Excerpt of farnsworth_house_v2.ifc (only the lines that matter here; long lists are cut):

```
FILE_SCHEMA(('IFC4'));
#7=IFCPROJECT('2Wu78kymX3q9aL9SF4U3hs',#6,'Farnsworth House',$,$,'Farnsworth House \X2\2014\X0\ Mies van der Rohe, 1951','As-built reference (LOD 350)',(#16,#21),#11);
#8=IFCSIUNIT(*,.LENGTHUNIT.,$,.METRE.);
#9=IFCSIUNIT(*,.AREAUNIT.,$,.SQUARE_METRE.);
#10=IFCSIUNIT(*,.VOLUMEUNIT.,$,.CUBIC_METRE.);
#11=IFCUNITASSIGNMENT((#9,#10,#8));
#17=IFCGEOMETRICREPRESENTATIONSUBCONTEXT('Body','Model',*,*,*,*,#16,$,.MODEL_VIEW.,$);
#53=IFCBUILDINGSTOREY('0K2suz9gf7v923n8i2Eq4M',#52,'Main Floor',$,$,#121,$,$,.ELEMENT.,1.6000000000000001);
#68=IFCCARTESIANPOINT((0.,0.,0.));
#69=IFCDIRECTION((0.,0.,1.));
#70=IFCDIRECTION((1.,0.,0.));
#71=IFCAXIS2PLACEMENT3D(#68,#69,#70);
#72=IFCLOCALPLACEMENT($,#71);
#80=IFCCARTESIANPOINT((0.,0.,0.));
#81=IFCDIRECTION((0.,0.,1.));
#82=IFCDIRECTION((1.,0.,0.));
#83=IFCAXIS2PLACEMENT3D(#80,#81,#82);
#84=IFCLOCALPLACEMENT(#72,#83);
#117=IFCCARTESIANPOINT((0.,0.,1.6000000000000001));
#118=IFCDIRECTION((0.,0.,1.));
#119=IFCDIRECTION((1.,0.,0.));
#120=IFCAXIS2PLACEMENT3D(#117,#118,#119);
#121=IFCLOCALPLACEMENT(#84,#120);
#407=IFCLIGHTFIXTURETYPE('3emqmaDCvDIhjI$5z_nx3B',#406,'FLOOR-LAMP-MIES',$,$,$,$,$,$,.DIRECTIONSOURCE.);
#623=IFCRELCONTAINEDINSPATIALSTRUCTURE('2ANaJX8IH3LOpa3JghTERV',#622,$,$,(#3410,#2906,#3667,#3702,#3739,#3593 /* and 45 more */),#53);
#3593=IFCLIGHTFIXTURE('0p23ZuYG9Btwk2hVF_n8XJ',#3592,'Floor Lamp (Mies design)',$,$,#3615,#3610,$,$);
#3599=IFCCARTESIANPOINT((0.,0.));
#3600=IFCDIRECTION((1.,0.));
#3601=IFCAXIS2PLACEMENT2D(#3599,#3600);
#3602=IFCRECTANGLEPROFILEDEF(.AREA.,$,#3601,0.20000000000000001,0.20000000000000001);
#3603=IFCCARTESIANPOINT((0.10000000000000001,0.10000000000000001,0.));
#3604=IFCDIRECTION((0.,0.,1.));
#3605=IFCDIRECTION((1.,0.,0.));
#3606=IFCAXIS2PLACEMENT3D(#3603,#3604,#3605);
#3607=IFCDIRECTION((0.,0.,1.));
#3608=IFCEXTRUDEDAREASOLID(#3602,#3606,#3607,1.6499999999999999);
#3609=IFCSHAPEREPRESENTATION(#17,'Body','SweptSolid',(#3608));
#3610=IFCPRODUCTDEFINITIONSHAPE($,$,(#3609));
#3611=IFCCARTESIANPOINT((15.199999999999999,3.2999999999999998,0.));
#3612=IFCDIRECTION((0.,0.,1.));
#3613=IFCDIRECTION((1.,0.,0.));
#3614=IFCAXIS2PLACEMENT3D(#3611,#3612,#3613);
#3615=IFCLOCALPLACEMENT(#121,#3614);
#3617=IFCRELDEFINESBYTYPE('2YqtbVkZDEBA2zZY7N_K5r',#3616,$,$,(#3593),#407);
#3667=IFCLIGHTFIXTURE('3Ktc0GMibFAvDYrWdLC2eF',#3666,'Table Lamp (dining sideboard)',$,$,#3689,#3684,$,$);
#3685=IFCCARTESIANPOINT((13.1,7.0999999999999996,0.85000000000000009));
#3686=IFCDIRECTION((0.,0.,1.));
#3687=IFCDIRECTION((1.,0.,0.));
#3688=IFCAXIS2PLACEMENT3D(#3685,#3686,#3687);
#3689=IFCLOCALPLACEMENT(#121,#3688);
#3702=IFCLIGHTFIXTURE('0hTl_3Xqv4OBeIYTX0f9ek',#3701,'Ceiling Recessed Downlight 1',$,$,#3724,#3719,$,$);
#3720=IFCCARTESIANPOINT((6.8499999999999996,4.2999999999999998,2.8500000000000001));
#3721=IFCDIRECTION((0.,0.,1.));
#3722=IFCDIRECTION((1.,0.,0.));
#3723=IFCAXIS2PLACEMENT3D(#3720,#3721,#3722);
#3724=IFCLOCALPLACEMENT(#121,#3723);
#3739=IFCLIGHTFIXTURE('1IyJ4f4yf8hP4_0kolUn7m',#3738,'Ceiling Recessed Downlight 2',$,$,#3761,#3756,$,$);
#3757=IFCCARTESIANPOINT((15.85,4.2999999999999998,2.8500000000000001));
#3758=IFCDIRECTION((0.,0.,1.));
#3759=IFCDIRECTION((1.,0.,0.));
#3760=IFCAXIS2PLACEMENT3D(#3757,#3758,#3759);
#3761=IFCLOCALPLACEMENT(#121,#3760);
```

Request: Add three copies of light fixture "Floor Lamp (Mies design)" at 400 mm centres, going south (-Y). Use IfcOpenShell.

```python
import numpy as np
import ifcopenshell
import ifcopenshell.api.geometry
import ifcopenshell.api.root
import ifcopenshell.util.element
import ifcopenshell.util.placement

model = ifcopenshell.open("farnsworth_house_v2.ifc")


def reuse_history(source, copy):
    """copy_class also copies each property set's owner history, people and application; keep the originals."""
    for rel in copy.IsDefinedBy:
        if rel.is_a("IfcRelDefinesByProperties") and (history := rel.RelatingPropertyDefinition.OwnerHistory):
            rel.RelatingPropertyDefinition.OwnerHistory = source.OwnerHistory
            ifcopenshell.util.element.remove_deep2(model, history)


source = model.by_guid("0p23ZuYG9Btwk2hVF_n8XJ")
base = ifcopenshell.util.placement.get_local_placement(source.ObjectPlacement)
step = np.array([0.0, -1.0, 0.0]) * 0.4

for i in range(1, 4):
    copy = ifcopenshell.api.root.copy_class(model, product=source)
    copy.Representation = ifcopenshell.util.element.copy_deep(
        model, source.Representation, exclude=["IfcGeometricRepresentationContext", "IfcRepresentationMap"]
    )
    reuse_history(source, copy)
    matrix = base.copy()
    matrix[:3, 3] += i * step
    print("added at", matrix[:3, 3].round(3) + 0.0)
    ifcopenshell.api.geometry.edit_object_placement(model, product=copy, matrix=matrix, is_si=False)

model.write("farnsworth_house_v2-out.ifc")
```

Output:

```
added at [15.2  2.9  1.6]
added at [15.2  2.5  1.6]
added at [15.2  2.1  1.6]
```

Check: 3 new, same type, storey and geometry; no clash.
